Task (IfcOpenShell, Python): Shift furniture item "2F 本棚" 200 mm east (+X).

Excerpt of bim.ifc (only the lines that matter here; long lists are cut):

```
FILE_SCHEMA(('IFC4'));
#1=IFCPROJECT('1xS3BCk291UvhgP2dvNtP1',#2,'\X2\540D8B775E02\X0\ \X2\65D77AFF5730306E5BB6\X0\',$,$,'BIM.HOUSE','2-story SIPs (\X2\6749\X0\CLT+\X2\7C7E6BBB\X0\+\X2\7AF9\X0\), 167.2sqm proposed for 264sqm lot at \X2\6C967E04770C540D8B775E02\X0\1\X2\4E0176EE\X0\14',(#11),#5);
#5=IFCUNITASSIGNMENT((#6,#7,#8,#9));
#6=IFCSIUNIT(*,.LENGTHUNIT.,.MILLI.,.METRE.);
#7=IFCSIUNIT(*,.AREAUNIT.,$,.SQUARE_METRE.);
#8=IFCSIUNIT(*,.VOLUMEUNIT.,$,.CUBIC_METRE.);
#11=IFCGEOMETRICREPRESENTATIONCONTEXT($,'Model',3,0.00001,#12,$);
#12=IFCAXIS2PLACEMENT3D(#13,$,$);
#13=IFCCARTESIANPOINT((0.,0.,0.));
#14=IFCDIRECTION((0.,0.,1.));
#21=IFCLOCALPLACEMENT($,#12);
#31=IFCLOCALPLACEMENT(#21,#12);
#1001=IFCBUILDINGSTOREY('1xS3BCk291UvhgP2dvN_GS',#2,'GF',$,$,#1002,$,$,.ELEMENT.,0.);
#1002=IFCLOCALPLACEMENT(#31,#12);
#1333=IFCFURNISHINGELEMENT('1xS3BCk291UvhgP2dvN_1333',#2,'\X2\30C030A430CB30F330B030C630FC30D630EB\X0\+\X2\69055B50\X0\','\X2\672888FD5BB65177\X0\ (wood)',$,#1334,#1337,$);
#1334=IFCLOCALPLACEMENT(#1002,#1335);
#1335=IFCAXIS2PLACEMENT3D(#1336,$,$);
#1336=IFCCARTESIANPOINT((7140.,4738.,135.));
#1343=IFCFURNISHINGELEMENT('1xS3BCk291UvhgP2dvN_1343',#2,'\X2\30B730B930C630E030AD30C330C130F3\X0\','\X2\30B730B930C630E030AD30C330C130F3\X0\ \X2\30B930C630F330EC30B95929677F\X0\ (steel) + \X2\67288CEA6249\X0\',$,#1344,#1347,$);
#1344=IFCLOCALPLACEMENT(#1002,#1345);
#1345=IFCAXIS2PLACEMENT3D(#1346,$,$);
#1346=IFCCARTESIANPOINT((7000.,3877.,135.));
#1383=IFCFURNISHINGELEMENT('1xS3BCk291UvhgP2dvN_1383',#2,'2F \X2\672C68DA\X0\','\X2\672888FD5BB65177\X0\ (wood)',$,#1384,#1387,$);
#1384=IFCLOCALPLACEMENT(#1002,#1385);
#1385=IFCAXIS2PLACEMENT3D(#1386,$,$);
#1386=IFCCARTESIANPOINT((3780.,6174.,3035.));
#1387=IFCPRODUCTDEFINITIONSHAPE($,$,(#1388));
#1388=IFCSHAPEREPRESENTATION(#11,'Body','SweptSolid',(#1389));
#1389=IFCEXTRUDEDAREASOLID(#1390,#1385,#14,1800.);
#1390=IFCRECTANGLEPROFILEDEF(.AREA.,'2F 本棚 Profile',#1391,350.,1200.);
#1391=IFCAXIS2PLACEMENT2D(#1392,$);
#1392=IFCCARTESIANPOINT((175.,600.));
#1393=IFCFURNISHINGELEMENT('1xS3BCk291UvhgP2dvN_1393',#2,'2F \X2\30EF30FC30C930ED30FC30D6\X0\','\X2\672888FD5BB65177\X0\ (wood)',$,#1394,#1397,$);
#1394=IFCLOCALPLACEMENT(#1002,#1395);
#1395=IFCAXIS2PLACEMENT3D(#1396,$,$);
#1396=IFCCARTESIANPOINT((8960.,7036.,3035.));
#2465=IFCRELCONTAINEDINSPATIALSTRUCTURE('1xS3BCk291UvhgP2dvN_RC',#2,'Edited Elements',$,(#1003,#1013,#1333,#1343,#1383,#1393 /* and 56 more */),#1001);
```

```python
import ifcopenshell
import ifcopenshell.api.geometry
import ifcopenshell.util.placement
import ifcopenshell.util.unit

model = ifcopenshell.open("bim.ifc")
unit_scale = ifcopenshell.util.unit.calculate_unit_scale(model)

item = model.by_guid("1xS3BCk291UvhgP2dvN_1383")
matrix = ifcopenshell.util.placement.get_local_placement(item.ObjectPlacement)
matrix[0, 3] += 0.2 / unit_scale
ifcopenshell.api.geometry.edit_object_placement(model, product=item, matrix=matrix, is_si=False)

print(ifcopenshell.util.placement.get_local_placement(item.ObjectPlacement).round(3) + 0.0)

model.write("bim_edited.ifc")
```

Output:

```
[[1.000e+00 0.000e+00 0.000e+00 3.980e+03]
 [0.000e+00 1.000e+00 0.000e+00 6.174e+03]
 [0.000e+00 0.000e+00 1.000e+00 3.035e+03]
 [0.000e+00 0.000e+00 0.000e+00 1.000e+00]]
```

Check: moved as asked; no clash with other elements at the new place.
